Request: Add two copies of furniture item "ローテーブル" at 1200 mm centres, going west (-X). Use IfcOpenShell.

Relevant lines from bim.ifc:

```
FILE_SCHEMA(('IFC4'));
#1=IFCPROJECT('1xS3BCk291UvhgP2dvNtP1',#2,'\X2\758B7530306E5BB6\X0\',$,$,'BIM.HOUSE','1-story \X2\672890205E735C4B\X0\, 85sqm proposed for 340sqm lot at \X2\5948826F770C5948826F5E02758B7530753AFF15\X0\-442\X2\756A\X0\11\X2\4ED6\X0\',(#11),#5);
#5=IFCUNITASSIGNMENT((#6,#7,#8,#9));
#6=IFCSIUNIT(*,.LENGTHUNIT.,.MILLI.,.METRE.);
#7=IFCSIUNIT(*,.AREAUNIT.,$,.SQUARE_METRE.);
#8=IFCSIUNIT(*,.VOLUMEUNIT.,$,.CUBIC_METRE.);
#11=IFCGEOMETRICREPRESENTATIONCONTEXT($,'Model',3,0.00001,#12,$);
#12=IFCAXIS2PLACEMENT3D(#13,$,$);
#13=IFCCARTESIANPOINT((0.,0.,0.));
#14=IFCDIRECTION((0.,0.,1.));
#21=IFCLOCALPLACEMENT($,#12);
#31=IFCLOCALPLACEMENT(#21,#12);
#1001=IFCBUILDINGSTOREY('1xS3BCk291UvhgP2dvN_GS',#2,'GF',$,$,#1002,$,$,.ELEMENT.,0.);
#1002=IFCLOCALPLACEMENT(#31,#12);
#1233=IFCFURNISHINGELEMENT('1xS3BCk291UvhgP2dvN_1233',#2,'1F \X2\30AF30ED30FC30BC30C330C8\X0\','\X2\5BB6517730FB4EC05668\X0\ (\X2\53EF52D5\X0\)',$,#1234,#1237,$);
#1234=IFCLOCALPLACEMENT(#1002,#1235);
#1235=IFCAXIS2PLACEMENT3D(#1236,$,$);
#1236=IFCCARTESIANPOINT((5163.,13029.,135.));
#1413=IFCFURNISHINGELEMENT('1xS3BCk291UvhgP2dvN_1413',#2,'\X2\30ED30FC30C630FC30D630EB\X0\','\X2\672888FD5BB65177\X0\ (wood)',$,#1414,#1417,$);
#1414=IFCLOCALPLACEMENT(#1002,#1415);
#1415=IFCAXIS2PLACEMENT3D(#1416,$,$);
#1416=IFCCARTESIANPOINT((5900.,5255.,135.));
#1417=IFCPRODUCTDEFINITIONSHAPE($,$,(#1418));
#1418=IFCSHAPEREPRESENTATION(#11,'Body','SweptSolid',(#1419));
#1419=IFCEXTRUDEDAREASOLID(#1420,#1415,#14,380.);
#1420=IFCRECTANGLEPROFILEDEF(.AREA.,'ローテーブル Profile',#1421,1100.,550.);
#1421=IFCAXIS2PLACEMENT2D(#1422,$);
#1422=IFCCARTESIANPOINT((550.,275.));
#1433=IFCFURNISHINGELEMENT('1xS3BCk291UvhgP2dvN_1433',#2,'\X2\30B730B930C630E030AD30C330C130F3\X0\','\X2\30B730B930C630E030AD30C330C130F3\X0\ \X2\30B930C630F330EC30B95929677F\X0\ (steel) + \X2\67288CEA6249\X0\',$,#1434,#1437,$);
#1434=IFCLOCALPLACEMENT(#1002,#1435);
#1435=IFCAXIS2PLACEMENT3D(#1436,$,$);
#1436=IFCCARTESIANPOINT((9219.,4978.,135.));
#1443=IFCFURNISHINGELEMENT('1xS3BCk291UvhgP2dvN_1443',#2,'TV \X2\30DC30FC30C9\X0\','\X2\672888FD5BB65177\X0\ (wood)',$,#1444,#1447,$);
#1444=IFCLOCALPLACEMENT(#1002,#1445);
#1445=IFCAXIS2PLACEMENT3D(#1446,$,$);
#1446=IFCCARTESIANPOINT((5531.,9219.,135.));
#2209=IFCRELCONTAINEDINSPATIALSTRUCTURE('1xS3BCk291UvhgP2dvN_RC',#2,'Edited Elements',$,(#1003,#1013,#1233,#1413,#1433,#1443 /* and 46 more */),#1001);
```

```python
import numpy as np
import ifcopenshell
import ifcopenshell.api.geometry
import ifcopenshell.api.root
import ifcopenshell.util.element
import ifcopenshell.util.placement
import ifcopenshell.util.unit

model = ifcopenshell.open("bim.ifc")
unit_scale = ifcopenshell.util.unit.calculate_unit_scale(model)


def reuse_history(source, copy):
    """copy_class also copies each property set's owner history, people and application; keep the originals."""
    for rel in copy.IsDefinedBy:
        if rel.is_a("IfcRelDefinesByProperties") and (history := rel.RelatingPropertyDefinition.OwnerHistory):
            rel.RelatingPropertyDefinition.OwnerHistory = source.OwnerHistory
            ifcopenshell.util.element.remove_deep2(model, history)


source = model.by_guid("1xS3BCk291UvhgP2dvN_1413")
base = ifcopenshell.util.placement.get_local_placement(source.ObjectPlacement)
step = np.array([-1.0, 0.0, 0.0]) * 1.2 / unit_scale

for i in range(1, 3):
    copy = ifcopenshell.api.root.copy_class(model, product=source)
    copy.Representation = ifcopenshell.util.element.copy_deep(
        model, source.Representation, exclude=["IfcGeometricRepresentationContext", "IfcRepresentationMap"]
    )
    reuse_history(source, copy)
    matrix = base.copy()
    matrix[:3, 3] += i * step
    print("added at", matrix[:3, 3].round(3) + 0.0)
    ifcopenshell.api.geometry.edit_object_placement(model, product=copy, matrix=matrix, is_si=False)

model.write("bim_rev.ifc")
```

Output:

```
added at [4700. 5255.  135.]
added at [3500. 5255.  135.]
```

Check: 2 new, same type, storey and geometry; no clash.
